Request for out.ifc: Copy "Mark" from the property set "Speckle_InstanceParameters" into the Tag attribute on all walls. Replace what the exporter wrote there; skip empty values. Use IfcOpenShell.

First a look at what the model holds.

```python
import ifcopenshell
import ifcopenshell.util.element

model = ifcopenshell.open("out.ifc")
print(model.schema)
walls = model.by_type("IfcWall")
print(len(walls), "walls")
for e in walls[:8]:
    source = ifcopenshell.util.element.get_pset(e, "Speckle_InstanceParameters", "Mark")
    target = e.Tag
    print(e.id(), repr(source), repr(target), sep=" | ")
```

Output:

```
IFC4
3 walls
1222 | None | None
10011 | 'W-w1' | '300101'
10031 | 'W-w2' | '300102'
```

```python
import ifcopenshell
import ifcopenshell.util.element

model = ifcopenshell.open("out.ifc")

count = 0
for e in model.by_type("IfcWall"):
    value = ifcopenshell.util.element.get_pset(e, "Speckle_InstanceParameters", "Mark")
    current = e.Tag
    if not value or not value.strip() or current == value:
        continue
    e.Tag = value
    count += 1

print(count, "walls updated")

model.write("out-out.ifc")
```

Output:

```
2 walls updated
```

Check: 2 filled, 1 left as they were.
